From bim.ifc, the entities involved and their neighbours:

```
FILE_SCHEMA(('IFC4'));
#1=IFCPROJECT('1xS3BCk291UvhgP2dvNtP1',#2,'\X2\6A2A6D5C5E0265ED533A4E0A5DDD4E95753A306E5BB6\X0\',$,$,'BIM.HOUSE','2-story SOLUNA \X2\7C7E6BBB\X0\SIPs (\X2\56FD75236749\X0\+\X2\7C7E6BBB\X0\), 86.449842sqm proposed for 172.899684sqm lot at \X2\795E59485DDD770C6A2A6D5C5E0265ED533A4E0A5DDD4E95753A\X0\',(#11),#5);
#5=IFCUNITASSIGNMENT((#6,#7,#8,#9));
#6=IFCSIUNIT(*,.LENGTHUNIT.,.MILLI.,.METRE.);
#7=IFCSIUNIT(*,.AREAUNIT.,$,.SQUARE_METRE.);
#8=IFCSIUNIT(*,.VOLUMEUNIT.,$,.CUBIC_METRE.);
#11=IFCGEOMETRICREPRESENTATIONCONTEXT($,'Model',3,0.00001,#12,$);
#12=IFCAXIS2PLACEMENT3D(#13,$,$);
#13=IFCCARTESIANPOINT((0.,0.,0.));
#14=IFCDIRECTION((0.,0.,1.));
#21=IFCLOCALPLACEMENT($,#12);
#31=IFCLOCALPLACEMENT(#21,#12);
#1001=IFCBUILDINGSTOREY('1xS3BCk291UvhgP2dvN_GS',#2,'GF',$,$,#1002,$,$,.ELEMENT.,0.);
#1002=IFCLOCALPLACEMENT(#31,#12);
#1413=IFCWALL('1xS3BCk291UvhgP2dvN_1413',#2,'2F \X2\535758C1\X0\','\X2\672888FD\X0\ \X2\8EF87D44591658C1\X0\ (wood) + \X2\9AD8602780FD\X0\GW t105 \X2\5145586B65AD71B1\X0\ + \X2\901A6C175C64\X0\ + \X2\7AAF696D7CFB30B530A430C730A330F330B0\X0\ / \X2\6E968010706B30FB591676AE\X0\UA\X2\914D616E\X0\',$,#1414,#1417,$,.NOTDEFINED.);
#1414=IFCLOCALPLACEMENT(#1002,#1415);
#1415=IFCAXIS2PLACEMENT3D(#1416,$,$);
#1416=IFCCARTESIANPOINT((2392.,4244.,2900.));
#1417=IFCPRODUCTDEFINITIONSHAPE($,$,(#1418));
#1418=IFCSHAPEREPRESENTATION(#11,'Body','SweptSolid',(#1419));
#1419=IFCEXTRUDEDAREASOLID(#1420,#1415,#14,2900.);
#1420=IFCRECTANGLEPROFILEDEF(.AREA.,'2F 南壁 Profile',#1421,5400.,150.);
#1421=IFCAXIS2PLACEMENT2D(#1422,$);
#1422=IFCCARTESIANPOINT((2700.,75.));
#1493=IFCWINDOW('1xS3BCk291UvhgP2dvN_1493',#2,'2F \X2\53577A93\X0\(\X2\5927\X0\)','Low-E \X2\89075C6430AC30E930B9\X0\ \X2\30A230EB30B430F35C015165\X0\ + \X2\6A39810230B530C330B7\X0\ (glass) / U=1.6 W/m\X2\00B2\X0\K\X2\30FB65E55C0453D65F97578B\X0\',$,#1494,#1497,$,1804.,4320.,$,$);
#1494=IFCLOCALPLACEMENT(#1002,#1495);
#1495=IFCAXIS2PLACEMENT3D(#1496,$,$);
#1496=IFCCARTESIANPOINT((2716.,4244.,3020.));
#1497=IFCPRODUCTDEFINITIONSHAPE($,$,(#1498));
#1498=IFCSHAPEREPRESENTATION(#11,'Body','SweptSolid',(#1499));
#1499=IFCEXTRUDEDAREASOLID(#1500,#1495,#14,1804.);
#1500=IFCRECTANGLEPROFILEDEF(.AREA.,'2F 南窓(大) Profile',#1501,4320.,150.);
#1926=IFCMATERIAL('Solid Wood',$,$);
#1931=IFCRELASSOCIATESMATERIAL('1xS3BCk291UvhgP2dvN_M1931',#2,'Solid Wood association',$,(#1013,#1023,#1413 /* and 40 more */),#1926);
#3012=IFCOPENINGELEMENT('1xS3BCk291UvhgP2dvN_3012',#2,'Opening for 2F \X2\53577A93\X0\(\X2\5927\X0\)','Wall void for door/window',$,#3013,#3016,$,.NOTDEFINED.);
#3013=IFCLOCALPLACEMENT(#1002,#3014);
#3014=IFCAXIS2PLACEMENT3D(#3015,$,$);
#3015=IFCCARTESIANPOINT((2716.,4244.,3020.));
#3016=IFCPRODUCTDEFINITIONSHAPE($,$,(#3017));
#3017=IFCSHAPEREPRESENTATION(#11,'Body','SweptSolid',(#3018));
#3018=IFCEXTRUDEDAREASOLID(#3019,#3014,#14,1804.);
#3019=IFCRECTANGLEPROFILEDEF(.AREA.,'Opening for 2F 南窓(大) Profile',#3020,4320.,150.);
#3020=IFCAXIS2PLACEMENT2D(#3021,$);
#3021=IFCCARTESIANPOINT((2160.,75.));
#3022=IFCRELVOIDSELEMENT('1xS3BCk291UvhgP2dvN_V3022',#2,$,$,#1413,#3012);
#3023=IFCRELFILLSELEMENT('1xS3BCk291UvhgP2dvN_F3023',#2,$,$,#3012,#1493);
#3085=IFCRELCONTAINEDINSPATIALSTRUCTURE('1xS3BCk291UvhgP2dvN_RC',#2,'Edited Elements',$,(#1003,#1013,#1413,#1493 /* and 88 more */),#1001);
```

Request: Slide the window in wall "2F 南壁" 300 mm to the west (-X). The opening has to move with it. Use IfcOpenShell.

```python
import ifcopenshell
import ifcopenshell.api.geometry
import ifcopenshell.util.placement
import ifcopenshell.util.unit

model = ifcopenshell.open("bim.ifc")
unit_scale = ifcopenshell.util.unit.calculate_unit_scale(model)

window = model.by_guid("1xS3BCk291UvhgP2dvN_1493")
opening = window.FillsVoids[0].RelatingOpeningElement
wall = opening.VoidsElements[0].RelatingBuildingElement

wall_matrix = ifcopenshell.util.placement.get_local_placement(wall.ObjectPlacement)
shift = wall_matrix[:3, 0] * -0.3 / unit_scale
before = ifcopenshell.util.placement.get_local_placement(window.ObjectPlacement)[:3, 3].copy()

# The window is not placed relative to its opening, so move both.
for product in (opening, window):
    matrix = ifcopenshell.util.placement.get_local_placement(product.ObjectPlacement)
    matrix[:3, 3] += shift
    ifcopenshell.api.geometry.edit_object_placement(model, product=product, matrix=matrix, is_si=False)

after = ifcopenshell.util.placement.get_local_placement(window.ObjectPlacement)[:3, 3]
print("window moved by", (after - before).round(3) + 0.0)

model.write("bim_updated.ifc")
```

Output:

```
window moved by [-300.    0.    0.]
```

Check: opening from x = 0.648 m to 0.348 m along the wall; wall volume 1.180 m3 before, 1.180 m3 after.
